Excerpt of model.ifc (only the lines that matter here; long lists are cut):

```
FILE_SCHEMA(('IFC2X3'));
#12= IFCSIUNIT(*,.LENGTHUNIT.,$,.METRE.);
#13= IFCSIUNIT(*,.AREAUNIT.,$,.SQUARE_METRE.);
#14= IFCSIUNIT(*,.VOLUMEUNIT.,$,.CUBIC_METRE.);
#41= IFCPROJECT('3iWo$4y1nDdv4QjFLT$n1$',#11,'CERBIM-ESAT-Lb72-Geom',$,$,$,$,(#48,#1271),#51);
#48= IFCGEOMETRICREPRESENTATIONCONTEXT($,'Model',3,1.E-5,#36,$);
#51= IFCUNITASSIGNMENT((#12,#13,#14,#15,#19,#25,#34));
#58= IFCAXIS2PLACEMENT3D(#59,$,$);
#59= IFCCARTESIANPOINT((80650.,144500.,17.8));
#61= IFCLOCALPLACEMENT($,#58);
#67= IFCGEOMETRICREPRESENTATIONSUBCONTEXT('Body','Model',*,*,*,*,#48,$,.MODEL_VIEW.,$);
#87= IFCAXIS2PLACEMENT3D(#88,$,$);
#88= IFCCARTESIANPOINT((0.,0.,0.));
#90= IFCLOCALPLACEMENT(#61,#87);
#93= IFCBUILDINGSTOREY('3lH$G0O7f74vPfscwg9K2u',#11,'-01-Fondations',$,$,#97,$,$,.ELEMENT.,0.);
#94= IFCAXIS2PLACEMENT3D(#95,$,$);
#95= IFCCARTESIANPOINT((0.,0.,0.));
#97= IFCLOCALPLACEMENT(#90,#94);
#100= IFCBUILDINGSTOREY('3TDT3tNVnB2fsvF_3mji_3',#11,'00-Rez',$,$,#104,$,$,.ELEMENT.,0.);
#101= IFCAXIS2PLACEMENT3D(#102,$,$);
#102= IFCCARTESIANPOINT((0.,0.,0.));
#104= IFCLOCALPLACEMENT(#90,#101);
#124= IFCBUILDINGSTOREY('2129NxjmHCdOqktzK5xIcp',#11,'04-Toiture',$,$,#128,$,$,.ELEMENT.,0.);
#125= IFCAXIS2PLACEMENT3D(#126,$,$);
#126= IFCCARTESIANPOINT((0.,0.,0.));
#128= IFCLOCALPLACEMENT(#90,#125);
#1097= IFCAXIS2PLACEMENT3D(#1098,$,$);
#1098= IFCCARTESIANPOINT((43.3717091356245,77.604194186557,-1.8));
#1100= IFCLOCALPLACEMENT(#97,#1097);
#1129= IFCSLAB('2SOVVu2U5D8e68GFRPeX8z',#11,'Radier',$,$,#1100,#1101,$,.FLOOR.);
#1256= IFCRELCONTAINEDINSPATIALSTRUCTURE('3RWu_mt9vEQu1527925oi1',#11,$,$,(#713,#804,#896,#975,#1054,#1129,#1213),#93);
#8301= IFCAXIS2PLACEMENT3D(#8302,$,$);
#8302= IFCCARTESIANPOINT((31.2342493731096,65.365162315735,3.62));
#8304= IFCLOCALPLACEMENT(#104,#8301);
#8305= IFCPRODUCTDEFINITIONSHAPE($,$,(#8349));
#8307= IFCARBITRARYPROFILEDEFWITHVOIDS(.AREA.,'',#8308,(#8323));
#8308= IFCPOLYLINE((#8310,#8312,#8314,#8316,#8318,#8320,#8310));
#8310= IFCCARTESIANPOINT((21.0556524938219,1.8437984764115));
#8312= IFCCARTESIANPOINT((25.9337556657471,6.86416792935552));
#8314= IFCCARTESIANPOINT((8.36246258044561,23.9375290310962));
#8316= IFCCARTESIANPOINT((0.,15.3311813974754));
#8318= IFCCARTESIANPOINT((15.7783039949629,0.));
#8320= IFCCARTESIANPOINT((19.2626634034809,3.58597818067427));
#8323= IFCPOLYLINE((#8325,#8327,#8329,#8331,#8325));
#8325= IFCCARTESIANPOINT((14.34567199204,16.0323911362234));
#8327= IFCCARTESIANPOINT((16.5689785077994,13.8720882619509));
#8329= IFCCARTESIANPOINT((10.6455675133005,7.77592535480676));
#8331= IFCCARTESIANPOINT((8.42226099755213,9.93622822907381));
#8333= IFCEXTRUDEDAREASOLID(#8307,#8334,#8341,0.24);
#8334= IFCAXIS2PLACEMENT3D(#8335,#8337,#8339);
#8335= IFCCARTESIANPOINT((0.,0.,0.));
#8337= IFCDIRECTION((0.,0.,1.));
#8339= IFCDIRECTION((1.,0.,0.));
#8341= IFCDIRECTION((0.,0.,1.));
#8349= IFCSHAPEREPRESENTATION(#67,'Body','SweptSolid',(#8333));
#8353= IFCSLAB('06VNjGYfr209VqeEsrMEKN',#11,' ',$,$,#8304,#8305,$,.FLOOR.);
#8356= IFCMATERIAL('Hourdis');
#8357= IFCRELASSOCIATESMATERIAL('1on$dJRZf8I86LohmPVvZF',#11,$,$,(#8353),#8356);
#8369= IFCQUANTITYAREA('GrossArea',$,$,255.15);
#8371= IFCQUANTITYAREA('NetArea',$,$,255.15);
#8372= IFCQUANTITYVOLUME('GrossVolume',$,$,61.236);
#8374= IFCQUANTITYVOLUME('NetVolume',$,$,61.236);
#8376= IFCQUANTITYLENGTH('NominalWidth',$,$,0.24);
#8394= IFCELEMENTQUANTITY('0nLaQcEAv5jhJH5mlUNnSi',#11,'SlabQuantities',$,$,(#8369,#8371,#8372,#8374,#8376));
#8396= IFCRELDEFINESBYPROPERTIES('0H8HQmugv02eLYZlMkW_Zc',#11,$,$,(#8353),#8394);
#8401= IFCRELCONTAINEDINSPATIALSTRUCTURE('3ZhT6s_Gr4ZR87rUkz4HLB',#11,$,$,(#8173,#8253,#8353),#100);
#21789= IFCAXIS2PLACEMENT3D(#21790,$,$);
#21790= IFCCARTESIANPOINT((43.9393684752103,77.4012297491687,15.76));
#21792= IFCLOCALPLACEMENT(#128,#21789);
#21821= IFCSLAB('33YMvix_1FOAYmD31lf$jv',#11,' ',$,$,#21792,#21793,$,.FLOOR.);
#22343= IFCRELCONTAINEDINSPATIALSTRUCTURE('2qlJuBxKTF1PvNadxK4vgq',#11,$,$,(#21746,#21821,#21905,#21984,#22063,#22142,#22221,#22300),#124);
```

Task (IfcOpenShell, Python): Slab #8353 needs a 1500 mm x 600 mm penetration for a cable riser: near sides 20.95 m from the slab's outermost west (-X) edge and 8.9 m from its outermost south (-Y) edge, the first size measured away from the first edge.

```python
import numpy as np
import ifcopenshell
import ifcopenshell.api.feature
import ifcopenshell.api.geometry
import ifcopenshell.api.pset
import ifcopenshell.api.root
import ifcopenshell.geom
import ifcopenshell.util.element
import ifcopenshell.util.placement
import ifcopenshell.util.representation
import ifcopenshell.util.shape
import ifcopenshell.util.unit

model = ifcopenshell.open("model.ifc")
unit_scale = ifcopenshell.util.unit.calculate_unit_scale(model)
area_scale = ifcopenshell.util.unit.calculate_unit_scale(model, "AREAUNIT")
volume_scale = ifcopenshell.util.unit.calculate_unit_scale(model, "VOLUMEUNIT")
settings = ifcopenshell.geom.settings()


def volume(element):
    """Net volume in cubic metres, openings subtracted."""
    shape = ifcopenshell.geom.create_shape(settings, element)
    return ifcopenshell.util.shape.get_volume(shape.geometry)


slab = model.by_guid("06VNjGYfr209VqeEsrMEKN")
before = volume(slab)

# Extent in the slab's own axes, in metres. The edges named are its -X and -Y sides.
slab_shape = ifcopenshell.geom.create_shape(settings, slab)
vertices = ifcopenshell.util.shape.get_vertices(slab_shape.geometry)
x_min, y_min, bottom = vertices.min(axis=0)
top = vertices[:, 2].max()

opening = ifcopenshell.api.root.create_entity(model, ifc_class="IfcOpeningElement", name="Cable riser opening")
context = ifcopenshell.util.representation.get_context(model, "Model", "Body", "MODEL_VIEW")
width, depth = 1.5, 0.6
outline = [(0.0, 0.0), (width, 0.0), (width, depth), (0.0, depth), (0.0, 0.0)]
# Overshoot both faces by 50 mm so the cut is clean.
shape = ifcopenshell.api.geometry.add_slab_representation(
    model, context=context, depth=top - bottom + 0.1, polyline=outline
)
ifcopenshell.api.geometry.assign_representation(model, product=opening, representation=shape)

matrix = ifcopenshell.util.placement.get_local_placement(slab.ObjectPlacement)
matrix[:, 3] = matrix @ np.append(np.array([x_min + 20.95, y_min + 8.9, bottom - 0.05]) / unit_scale, 1.0)
ifcopenshell.api.geometry.edit_object_placement(model, product=opening, matrix=matrix, is_si=False)
ifcopenshell.api.feature.add_feature(model, feature=opening, element=slab)

after = volume(slab)

# Update the slab's stored quantities.
qto = model.by_id(ifcopenshell.util.element.get_pset(slab, "SlabQuantities", should_inherit=False)["id"])
ifcopenshell.api.pset.edit_qto(model, qto=qto, properties={
    "NetArea": after / (top - bottom) / area_scale,
    "NetVolume": after / volume_scale,
})

print(f"slab volume {before:.3f} -> {after:.3f} m3")

model.write("model-out.ifc")
```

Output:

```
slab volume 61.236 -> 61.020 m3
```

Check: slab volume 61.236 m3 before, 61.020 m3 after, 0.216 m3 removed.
